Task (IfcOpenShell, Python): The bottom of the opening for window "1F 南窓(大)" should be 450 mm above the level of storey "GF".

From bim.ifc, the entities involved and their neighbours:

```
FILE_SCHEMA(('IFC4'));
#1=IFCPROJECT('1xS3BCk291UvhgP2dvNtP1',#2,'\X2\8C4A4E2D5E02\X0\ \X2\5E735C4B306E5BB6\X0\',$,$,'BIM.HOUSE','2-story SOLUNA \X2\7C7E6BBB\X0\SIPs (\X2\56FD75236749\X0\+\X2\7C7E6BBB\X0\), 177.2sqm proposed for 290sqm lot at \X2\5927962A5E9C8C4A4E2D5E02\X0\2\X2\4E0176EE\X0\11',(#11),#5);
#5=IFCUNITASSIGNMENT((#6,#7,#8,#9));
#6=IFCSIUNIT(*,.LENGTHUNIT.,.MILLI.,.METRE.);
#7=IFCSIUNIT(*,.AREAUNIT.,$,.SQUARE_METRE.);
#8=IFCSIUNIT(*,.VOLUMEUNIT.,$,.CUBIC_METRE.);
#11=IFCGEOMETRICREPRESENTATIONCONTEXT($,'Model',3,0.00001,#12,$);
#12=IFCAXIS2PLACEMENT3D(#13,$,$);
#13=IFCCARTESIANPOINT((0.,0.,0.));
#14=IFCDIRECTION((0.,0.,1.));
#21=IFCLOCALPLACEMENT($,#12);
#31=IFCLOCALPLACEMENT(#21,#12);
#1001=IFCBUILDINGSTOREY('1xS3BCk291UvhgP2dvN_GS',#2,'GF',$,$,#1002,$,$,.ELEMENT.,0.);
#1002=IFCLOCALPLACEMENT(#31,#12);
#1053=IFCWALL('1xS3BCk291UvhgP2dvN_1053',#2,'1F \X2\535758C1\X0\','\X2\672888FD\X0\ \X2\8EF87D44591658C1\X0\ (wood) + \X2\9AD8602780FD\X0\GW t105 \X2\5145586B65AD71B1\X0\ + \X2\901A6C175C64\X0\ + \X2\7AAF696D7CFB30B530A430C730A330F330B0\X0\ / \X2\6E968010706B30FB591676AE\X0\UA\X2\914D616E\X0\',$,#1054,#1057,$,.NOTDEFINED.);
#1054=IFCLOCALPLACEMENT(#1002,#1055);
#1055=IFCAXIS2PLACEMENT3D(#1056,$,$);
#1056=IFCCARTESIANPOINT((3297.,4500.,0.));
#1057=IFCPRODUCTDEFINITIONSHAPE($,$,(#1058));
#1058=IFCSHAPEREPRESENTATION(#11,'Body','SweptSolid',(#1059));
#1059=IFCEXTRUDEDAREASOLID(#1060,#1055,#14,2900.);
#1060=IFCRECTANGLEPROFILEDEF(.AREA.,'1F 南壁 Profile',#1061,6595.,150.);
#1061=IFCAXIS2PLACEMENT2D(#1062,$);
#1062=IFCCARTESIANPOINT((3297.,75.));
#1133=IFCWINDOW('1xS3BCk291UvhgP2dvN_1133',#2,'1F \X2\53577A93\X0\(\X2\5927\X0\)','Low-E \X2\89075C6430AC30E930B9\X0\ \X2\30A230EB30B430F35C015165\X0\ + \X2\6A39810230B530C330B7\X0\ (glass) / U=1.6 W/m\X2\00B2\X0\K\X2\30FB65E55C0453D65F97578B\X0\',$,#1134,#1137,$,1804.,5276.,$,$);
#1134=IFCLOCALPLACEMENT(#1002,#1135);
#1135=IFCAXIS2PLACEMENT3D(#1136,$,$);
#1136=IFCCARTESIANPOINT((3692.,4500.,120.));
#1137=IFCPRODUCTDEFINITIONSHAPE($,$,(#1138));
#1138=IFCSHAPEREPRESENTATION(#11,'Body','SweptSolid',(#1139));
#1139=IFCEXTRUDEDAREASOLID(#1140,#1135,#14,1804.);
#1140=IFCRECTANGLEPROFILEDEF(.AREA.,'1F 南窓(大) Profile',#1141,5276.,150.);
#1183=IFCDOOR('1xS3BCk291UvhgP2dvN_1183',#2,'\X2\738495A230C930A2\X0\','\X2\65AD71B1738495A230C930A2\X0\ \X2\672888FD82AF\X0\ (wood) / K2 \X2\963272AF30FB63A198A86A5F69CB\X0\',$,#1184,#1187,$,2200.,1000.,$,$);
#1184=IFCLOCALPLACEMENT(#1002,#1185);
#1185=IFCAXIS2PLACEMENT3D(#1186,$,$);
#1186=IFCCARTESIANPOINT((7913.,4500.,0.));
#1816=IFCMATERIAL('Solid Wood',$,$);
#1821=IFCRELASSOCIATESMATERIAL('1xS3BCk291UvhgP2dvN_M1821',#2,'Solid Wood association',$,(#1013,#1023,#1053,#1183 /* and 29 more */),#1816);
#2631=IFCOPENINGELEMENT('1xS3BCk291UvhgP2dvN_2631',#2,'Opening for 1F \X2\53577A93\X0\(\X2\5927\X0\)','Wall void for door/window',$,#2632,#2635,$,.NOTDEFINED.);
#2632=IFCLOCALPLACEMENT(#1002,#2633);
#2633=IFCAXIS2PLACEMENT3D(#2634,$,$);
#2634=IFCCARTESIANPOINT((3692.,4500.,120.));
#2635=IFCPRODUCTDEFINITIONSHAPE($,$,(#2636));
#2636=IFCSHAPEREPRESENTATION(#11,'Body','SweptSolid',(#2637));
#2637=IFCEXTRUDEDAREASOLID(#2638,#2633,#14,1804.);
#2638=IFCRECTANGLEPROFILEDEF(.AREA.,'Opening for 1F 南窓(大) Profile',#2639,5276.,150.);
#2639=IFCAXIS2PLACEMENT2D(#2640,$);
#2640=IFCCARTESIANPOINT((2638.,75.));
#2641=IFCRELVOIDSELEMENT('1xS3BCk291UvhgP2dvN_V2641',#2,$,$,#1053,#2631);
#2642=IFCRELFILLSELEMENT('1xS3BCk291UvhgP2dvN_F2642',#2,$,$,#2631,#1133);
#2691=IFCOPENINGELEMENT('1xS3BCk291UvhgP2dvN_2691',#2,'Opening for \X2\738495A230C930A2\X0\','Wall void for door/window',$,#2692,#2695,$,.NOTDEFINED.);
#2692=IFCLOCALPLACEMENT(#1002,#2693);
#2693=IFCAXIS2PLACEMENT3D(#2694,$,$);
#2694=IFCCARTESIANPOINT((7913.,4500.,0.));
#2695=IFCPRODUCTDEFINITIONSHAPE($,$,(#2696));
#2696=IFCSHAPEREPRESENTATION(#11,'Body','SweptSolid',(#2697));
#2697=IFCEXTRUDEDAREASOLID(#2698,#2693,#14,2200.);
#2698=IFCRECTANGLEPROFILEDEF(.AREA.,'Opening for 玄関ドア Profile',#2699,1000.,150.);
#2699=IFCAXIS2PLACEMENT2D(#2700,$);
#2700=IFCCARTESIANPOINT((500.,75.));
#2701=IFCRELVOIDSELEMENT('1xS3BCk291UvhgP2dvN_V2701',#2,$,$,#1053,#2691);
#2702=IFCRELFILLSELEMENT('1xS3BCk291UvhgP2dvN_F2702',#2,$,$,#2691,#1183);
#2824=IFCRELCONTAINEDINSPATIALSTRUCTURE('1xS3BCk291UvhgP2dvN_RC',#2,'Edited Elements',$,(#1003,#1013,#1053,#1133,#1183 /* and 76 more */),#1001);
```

```python
import numpy as np
import ifcopenshell
import ifcopenshell.api.geometry
import ifcopenshell.geom
import ifcopenshell.util.element
import ifcopenshell.util.placement
import ifcopenshell.util.shape
import ifcopenshell.util.unit

model = ifcopenshell.open("bim.ifc")
unit_scale = ifcopenshell.util.unit.calculate_unit_scale(model)

window = model.by_guid("1xS3BCk291UvhgP2dvN_1133")
opening = window.FillsVoids[0].RelatingOpeningElement
storey = ifcopenshell.util.element.get_container(window, ifc_class="IfcBuildingStorey")
level = ifcopenshell.util.placement.get_local_placement(storey.ObjectPlacement)[2, 3]

# The opening's origin need not be at the sill, so measure its lowest point.
shape = ifcopenshell.geom.create_shape(ifcopenshell.geom.settings(), opening)
bottom = ifcopenshell.util.shape.get_shape_bottom_elevation(shape, shape.geometry) / unit_scale
dz = level + 450.0 - bottom

shift = np.array([0.0, 0.0, dz])
# The window is not placed relative to its opening, so move both.
for product in (opening, window):
    matrix = ifcopenshell.util.placement.get_local_placement(product.ObjectPlacement)
    matrix[:3, 3] += shift
    ifcopenshell.api.geometry.edit_object_placement(model, product=product, matrix=matrix, is_si=False)

print(f"moved by {dz * unit_scale:+.3f} m")

model.write("bim-out.ifc")
```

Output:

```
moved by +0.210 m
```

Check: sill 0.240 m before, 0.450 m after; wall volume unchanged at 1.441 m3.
